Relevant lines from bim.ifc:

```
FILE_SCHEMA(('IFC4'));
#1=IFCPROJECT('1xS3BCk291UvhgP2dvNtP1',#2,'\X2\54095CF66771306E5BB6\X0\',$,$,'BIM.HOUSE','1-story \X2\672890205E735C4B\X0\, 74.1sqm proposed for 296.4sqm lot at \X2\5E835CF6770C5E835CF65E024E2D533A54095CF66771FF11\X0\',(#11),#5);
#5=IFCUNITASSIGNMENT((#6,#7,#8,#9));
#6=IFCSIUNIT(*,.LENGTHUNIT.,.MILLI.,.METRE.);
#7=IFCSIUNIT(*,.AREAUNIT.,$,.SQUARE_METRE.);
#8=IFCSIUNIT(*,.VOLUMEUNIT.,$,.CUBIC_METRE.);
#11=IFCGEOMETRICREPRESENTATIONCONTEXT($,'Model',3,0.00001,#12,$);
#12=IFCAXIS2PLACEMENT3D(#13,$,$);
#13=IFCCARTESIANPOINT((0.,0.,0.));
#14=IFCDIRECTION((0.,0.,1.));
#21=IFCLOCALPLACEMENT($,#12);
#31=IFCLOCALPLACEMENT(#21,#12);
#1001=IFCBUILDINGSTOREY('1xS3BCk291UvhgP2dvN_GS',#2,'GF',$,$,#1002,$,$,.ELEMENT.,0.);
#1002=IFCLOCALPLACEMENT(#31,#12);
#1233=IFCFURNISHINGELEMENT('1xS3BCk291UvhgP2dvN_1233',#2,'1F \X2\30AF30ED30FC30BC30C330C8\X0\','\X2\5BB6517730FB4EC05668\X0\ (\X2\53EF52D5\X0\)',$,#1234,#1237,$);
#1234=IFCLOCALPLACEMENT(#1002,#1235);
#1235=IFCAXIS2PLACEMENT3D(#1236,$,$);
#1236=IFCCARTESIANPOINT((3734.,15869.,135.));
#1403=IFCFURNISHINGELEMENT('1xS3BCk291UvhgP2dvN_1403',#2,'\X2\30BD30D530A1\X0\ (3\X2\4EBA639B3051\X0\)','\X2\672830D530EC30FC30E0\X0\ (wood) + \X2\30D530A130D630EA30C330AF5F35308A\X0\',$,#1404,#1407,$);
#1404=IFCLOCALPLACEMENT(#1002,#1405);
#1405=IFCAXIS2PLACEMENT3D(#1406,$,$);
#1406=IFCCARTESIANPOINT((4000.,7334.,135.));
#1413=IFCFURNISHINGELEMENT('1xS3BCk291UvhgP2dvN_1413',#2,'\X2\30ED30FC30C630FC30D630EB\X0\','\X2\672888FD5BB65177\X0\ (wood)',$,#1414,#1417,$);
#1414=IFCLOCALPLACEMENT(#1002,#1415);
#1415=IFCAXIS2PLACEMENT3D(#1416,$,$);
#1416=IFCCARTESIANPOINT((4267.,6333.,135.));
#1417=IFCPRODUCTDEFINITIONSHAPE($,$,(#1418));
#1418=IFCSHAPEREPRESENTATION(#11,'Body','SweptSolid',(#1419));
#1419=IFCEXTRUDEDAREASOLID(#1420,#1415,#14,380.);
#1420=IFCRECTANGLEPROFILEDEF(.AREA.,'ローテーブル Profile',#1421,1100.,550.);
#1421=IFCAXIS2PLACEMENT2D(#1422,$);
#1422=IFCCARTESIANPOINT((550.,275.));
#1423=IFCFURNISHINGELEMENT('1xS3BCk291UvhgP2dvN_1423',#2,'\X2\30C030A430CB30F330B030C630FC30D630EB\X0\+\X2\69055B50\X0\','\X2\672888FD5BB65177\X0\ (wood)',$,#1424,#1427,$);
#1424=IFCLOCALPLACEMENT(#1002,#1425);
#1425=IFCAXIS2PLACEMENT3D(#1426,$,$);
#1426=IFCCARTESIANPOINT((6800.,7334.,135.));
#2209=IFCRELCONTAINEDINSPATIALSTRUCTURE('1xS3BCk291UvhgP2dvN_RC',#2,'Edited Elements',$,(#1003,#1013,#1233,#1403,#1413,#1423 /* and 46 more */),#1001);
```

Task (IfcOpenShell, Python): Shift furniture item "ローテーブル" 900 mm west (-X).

```python
import ifcopenshell
import ifcopenshell.api.geometry
import ifcopenshell.util.placement
import ifcopenshell.util.unit

model = ifcopenshell.open("bim.ifc")
unit_scale = ifcopenshell.util.unit.calculate_unit_scale(model)

item = model.by_id(1413)
matrix = ifcopenshell.util.placement.get_local_placement(item.ObjectPlacement)
matrix[0, 3] -= 0.9 / unit_scale
ifcopenshell.api.geometry.edit_object_placement(model, product=item, matrix=matrix, is_si=False)

print(ifcopenshell.util.placement.get_local_placement(item.ObjectPlacement).round(3) + 0.0)

model.write("bim_edited.ifc")
```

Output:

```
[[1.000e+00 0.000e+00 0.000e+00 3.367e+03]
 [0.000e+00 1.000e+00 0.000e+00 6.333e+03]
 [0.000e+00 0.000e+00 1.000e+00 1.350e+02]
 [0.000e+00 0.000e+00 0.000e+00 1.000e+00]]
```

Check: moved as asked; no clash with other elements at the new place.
